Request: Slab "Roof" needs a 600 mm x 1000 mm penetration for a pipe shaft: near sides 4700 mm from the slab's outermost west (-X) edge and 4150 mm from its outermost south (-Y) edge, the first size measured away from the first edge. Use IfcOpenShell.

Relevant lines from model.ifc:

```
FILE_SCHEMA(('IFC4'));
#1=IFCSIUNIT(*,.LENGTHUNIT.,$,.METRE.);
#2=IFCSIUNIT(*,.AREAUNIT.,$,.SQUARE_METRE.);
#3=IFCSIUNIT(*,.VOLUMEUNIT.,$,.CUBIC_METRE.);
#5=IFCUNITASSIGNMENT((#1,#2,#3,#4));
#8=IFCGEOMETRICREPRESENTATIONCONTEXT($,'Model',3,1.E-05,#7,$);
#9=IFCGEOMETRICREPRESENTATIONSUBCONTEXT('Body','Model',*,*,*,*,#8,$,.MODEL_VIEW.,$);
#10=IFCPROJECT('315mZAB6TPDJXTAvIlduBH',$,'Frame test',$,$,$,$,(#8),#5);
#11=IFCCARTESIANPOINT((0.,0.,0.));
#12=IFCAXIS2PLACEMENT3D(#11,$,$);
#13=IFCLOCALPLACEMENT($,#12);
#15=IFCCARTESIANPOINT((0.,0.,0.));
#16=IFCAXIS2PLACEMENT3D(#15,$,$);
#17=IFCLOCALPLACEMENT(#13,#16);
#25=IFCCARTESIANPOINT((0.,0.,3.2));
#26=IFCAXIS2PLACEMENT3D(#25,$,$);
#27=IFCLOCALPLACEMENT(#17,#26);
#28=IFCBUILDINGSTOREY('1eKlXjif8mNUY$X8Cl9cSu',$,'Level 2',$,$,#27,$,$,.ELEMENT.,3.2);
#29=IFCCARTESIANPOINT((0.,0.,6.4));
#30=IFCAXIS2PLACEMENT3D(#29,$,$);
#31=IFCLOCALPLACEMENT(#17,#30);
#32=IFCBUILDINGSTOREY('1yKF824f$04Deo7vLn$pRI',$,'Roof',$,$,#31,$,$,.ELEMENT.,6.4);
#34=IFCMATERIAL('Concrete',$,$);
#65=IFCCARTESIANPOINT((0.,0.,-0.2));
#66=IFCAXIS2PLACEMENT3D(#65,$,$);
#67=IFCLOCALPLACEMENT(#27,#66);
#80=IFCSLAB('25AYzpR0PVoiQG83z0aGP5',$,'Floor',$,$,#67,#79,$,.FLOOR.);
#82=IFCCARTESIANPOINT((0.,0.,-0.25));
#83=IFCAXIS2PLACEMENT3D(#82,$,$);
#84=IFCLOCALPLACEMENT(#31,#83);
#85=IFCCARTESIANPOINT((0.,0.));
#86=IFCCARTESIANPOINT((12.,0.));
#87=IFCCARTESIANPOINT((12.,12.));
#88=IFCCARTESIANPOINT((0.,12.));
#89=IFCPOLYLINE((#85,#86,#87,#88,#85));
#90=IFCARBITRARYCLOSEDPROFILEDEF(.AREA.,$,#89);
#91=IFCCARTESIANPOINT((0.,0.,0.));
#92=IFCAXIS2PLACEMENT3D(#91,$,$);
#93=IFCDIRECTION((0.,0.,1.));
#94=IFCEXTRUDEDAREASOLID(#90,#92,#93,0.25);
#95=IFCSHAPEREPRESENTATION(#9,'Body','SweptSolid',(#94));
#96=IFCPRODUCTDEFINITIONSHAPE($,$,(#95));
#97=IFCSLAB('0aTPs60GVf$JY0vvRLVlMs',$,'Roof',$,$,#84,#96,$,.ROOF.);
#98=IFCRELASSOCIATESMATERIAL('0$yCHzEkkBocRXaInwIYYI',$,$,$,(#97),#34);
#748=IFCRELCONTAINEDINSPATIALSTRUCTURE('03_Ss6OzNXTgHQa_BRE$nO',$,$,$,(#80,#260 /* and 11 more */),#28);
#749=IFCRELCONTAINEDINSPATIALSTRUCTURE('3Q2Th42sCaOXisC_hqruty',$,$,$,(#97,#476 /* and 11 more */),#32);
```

```python
import numpy as np
import ifcopenshell
import ifcopenshell.api.feature
import ifcopenshell.api.geometry
import ifcopenshell.api.root
import ifcopenshell.geom
import ifcopenshell.util.placement
import ifcopenshell.util.representation
import ifcopenshell.util.shape
import ifcopenshell.util.unit

model = ifcopenshell.open("model.ifc")
unit_scale = ifcopenshell.util.unit.calculate_unit_scale(model)
settings = ifcopenshell.geom.settings()


def volume(element):
    """Net volume in cubic metres, openings subtracted."""
    shape = ifcopenshell.geom.create_shape(settings, element)
    return ifcopenshell.util.shape.get_volume(shape.geometry)


slab = model.by_guid("0aTPs60GVf$JY0vvRLVlMs")
before = volume(slab)

# Extent in the slab's own axes, in metres. The edges named are its -X and -Y sides.
slab_shape = ifcopenshell.geom.create_shape(settings, slab)
vertices = ifcopenshell.util.shape.get_vertices(slab_shape.geometry)
x_min, y_min, bottom = vertices.min(axis=0)
top = vertices[:, 2].max()

opening = ifcopenshell.api.root.create_entity(model, ifc_class="IfcOpeningElement", name="Pipe shaft opening", predefined_type="OPENING")
context = ifcopenshell.util.representation.get_context(model, "Model", "Body", "MODEL_VIEW")
width, depth = 0.6, 1
outline = [(0.0, 0.0), (width, 0.0), (width, depth), (0.0, depth), (0.0, 0.0)]
# Overshoot both faces by 50 mm so the cut is clean.
shape = ifcopenshell.api.geometry.add_slab_representation(
    model, context=context, depth=top - bottom + 0.1, polyline=outline
)
ifcopenshell.api.geometry.assign_representation(model, product=opening, representation=shape)

matrix = ifcopenshell.util.placement.get_local_placement(slab.ObjectPlacement)
matrix[:, 3] = matrix @ np.append(np.array([x_min + 4.7, y_min + 4.15, bottom - 0.05]) / unit_scale, 1.0)
ifcopenshell.api.geometry.edit_object_placement(model, product=opening, matrix=matrix, is_si=False)
ifcopenshell.api.feature.add_feature(model, feature=opening, element=slab)

after = volume(slab)

print(f"slab volume {before:.3f} -> {after:.3f} m3")

model.write("model_updated.ifc")
```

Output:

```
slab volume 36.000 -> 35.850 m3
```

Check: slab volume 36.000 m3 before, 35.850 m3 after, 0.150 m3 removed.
